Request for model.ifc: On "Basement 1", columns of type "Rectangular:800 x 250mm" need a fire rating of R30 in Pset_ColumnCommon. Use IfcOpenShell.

First a look at what the model holds.

```python
import ifcopenshell
import ifcopenshell.util.element

model = ifcopenshell.open("model.ifc")
print(model.schema)
storey = next(s for s in model.by_type("IfcBuildingStorey") if s.Name == "Basement 1")
columns = [e for e in ifcopenshell.util.element.get_decomposition(storey) if e.is_a("IfcColumn")]
seen = {}
for e in columns:
    element_type = ifcopenshell.util.element.get_type(e)
    key = (element_type.Name if element_type != e and element_type else None, ifcopenshell.util.element.get_pset(e, "Pset_ColumnCommon", "FireRating"))
    seen[key] = seen.get(key, 0) + 1
for (name, value), count in sorted(seen.items(), key=str):
    print(count, "x", name, "|", value)
```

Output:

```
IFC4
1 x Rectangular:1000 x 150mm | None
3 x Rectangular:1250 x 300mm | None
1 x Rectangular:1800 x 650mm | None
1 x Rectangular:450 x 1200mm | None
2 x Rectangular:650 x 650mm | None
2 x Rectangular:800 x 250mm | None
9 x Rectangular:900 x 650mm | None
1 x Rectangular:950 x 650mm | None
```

```python
import ifcopenshell
import ifcopenshell.api.pset
import ifcopenshell.util.element

model = ifcopenshell.open("model.ifc")

storey = next(s for s in model.by_type("IfcBuildingStorey") if s.Name == "Basement 1")
columns = [e for e in ifcopenshell.util.element.get_decomposition(storey) if e.is_a("IfcColumn")]

count = 0
for e in columns:
    element_type = ifcopenshell.util.element.get_type(e)
    if element_type in (None, e) or element_type.Name != "Rectangular:800 x 250mm":
        continue
    # add_pset returns the element's existing set when there is one.
    pset = ifcopenshell.api.pset.add_pset(model, product=e, name="Pset_ColumnCommon")
    ifcopenshell.api.pset.edit_pset(model, pset=pset, properties={"FireRating": "R30"})
    count += 1

print(count, "columns updated")

model.write("model_v2.ifc")
```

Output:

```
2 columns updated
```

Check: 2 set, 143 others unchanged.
